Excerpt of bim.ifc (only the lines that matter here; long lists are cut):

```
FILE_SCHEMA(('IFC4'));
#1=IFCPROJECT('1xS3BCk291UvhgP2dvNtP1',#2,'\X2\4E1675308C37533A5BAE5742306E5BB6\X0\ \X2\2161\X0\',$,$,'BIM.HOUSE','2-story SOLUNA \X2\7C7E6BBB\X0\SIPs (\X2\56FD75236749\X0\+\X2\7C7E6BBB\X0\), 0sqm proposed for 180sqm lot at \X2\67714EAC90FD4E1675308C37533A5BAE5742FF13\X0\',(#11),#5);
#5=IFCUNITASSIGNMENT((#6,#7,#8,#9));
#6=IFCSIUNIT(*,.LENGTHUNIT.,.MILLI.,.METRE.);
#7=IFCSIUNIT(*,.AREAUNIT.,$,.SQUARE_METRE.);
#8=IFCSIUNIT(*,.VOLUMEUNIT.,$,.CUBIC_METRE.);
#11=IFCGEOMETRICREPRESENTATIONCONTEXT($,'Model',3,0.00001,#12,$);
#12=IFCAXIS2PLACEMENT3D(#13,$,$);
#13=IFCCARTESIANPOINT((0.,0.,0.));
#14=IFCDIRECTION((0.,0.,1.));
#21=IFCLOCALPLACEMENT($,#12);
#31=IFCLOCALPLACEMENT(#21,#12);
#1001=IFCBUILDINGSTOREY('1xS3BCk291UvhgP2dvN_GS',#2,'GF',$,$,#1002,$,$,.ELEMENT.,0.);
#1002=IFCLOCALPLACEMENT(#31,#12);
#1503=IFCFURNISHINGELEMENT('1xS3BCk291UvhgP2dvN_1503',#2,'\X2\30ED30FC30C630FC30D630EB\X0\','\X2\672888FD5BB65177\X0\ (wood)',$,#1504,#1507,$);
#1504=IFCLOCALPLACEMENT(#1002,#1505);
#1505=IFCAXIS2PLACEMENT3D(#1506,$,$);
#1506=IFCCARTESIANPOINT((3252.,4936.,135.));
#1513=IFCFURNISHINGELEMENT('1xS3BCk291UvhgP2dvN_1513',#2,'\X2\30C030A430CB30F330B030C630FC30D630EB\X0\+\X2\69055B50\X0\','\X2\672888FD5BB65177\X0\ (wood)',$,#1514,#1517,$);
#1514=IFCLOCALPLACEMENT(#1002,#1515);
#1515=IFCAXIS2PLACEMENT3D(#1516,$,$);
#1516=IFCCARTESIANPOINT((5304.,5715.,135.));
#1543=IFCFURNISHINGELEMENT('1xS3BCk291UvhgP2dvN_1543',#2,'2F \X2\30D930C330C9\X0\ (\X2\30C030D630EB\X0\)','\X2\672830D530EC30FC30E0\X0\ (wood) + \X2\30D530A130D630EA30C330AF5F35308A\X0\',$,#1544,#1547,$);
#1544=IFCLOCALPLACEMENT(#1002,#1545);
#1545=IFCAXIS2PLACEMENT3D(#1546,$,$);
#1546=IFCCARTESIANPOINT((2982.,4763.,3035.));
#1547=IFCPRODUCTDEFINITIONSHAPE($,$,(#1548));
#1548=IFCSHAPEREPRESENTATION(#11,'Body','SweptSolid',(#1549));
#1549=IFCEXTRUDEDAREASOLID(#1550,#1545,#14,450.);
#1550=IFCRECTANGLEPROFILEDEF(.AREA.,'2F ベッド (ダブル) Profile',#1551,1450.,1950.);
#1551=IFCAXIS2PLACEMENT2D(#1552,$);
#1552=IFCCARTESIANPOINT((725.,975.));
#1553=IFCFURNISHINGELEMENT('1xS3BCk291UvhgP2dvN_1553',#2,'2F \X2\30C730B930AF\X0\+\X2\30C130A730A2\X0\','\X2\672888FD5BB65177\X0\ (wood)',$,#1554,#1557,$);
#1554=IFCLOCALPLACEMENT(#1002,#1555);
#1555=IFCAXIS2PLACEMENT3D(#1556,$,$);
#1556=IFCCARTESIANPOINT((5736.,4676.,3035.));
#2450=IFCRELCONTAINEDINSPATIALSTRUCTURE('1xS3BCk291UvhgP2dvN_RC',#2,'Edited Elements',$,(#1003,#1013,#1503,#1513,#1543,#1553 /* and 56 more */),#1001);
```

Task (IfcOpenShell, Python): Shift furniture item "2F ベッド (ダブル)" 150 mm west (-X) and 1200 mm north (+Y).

```python
import ifcopenshell
import ifcopenshell.api.geometry
import ifcopenshell.util.placement
import ifcopenshell.util.unit

model = ifcopenshell.open("bim.ifc")
unit_scale = ifcopenshell.util.unit.calculate_unit_scale(model)

item = model.by_guid("1xS3BCk291UvhgP2dvN_1543")
matrix = ifcopenshell.util.placement.get_local_placement(item.ObjectPlacement)
matrix[0, 3] -= 0.15 / unit_scale
matrix[1, 3] += 1.2 / unit_scale
ifcopenshell.api.geometry.edit_object_placement(model, product=item, matrix=matrix, is_si=False)

print(ifcopenshell.util.placement.get_local_placement(item.ObjectPlacement).round(3) + 0.0)

model.write("bim_v2.ifc")
```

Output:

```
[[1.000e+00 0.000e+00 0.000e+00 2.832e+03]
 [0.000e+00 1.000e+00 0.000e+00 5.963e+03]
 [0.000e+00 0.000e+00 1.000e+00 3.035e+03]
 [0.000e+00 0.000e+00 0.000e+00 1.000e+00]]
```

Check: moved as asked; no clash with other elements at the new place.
